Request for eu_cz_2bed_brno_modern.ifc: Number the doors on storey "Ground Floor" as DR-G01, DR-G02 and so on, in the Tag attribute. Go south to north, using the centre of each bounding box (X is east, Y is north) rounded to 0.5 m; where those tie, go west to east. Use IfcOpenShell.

First a look at what the model holds.

```python
import ifcopenshell
import ifcopenshell.util.element
import ifcopenshell.util.placement

model = ifcopenshell.open("eu_cz_2bed_brno_modern.ifc")
print(model.schema)
storey = next(s for s in model.by_type("IfcBuildingStorey") if s.Name == "Ground Floor")
doors = [e for e in ifcopenshell.util.element.get_decomposition(storey) if e.is_a("IfcDoor")]
for e in sorted(doors, key=lambda e: e.id()):
    origin = ifcopenshell.util.placement.get_local_placement(e.ObjectPlacement)[:3, 3]
    print(e.id(), e.Tag, e.Name, origin.round(2) + 0.0, sep=" | ")
```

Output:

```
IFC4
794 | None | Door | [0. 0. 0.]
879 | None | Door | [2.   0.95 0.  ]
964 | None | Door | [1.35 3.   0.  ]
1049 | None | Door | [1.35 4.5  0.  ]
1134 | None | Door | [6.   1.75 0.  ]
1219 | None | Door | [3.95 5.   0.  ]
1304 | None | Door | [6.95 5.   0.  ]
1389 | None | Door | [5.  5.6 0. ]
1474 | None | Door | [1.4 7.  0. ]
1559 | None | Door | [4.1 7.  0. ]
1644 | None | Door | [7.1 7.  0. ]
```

```python
import ifcopenshell
import ifcopenshell.geom
import ifcopenshell.util.element
import ifcopenshell.util.shape

model = ifcopenshell.open("eu_cz_2bed_brno_modern.ifc")
settings = ifcopenshell.geom.settings()
settings.set("use-world-coords", True)


def centre(element):
    shape = ifcopenshell.geom.create_shape(settings, element)
    return ifcopenshell.util.shape.get_bbox_centroid(shape.geometry)


storey = next(s for s in model.by_type("IfcBuildingStorey") if s.Name == "Ground Floor")
doors = [e for e in ifcopenshell.util.element.get_decomposition(storey) if e.is_a("IfcDoor")]

# Insertion points can sit at a corner or the storey origin, so sort by the geometry (in metres).
centres = {e: centre(e) for e in doors}
doors.sort(key=lambda e: (round(centres[e][1] / 0.5), centres[e][0]))

for i, e in enumerate(doors, start=1):
    number = f"DR-G{i:02d}"
    e.Tag = number
    print(e.id(), number)

model.write("eu_cz_2bed_brno_modern_rev.ifc")
```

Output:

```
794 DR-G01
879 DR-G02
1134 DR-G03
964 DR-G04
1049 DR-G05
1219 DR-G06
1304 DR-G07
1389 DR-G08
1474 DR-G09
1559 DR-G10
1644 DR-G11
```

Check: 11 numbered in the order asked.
